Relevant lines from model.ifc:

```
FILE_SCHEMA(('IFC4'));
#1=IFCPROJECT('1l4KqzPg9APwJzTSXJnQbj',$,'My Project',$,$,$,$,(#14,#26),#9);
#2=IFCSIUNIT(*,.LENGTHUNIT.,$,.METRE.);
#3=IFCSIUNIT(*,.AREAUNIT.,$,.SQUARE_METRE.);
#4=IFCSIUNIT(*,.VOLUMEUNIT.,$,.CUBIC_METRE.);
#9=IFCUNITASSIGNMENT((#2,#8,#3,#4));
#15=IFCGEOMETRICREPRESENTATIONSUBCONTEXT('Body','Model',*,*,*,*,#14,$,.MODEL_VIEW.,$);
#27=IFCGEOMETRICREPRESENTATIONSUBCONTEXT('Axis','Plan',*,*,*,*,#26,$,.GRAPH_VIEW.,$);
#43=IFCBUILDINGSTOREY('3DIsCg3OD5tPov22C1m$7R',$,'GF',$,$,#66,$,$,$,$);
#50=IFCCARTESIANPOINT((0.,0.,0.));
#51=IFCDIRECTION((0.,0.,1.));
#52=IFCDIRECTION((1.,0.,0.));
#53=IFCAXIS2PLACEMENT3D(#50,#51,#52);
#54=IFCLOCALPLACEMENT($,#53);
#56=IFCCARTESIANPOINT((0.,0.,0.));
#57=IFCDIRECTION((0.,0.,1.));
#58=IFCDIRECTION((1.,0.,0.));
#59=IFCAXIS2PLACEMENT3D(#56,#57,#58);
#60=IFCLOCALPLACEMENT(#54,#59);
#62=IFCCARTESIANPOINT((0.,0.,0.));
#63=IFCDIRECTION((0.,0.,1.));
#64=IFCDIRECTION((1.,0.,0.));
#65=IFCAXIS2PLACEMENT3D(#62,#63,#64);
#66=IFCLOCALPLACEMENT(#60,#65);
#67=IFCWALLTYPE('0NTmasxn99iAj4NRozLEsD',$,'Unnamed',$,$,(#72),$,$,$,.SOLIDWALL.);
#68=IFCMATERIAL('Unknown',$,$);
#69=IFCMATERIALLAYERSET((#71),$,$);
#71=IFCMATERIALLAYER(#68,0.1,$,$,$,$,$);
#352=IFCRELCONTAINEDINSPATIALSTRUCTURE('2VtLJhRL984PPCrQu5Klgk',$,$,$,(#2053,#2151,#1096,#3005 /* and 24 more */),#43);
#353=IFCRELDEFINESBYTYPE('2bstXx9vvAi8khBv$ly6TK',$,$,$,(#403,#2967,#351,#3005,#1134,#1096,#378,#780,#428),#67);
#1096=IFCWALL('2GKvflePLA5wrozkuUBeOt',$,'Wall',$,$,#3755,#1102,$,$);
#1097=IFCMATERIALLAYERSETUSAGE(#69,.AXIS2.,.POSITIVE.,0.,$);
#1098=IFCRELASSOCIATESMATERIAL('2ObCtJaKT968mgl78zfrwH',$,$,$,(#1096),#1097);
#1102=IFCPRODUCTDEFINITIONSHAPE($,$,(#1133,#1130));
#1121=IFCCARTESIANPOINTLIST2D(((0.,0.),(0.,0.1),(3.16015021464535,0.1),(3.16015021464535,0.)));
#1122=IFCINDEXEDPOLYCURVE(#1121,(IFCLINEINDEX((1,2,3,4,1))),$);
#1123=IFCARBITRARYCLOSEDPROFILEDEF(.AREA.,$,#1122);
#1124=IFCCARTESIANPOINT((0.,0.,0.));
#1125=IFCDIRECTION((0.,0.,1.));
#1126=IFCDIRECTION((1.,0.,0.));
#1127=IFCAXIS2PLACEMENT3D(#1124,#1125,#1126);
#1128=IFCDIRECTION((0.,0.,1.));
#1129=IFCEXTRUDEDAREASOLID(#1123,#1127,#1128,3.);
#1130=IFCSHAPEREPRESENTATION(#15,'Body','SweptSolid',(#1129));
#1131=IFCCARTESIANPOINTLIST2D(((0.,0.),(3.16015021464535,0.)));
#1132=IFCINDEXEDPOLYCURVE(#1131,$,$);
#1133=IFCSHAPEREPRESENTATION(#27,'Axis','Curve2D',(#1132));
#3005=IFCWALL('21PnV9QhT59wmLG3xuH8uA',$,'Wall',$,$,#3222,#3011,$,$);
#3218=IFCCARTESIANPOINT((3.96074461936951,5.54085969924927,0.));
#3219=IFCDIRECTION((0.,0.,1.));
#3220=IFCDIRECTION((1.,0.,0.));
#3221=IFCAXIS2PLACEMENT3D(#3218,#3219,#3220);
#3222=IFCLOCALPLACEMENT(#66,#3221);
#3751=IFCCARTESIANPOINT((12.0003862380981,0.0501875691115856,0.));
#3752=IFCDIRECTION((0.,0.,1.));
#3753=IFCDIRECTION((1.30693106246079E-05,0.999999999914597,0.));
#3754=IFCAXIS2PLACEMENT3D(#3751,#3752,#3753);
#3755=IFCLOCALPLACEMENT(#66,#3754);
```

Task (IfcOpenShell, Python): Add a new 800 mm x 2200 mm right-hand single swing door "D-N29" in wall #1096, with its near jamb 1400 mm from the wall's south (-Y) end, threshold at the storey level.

```python
import numpy as np
import ifcopenshell
import ifcopenshell.api.feature
import ifcopenshell.api.geometry
import ifcopenshell.api.root
import ifcopenshell.api.spatial
import ifcopenshell.geom
import ifcopenshell.util.element
import ifcopenshell.util.placement
import ifcopenshell.util.representation
import ifcopenshell.util.shape
import ifcopenshell.util.unit

model = ifcopenshell.open("model.ifc")
unit_scale = ifcopenshell.util.unit.calculate_unit_scale(model)
settings = ifcopenshell.geom.settings()


def volume(element):
    """Net volume in cubic metres, openings subtracted."""
    shape = ifcopenshell.geom.create_shape(settings, element)
    return ifcopenshell.util.shape.get_volume(shape.geometry)


wall = model.by_id(1096)
storey = ifcopenshell.util.element.get_container(wall, ifc_class="IfcBuildingStorey")
context = ifcopenshell.util.representation.get_context(model, "Model", "Body", "MODEL_VIEW")
before = volume(wall)

width, height, from_end, sill = 0.8, 2.2, 1.4, 0.0  # metres

# The wall runs along its own X axis, and the end named is its -X end.
wall_shape = ifcopenshell.geom.create_shape(settings, wall)
x, y, z = ifcopenshell.util.shape.get_vertices(wall_shape.geometry).T
start = x.min() + from_end
face, thickness = float(y.min()), float(y.max() - y.min())
wall_matrix = ifcopenshell.util.placement.get_local_placement(wall.ObjectPlacement)
level = ifcopenshell.util.placement.get_local_placement(storey.ObjectPlacement)[2, 3]


def in_wall(x, y):
    """Placement at x, y metres in the wall's axes, at sill height."""
    matrix = wall_matrix.copy()
    matrix[:, 3] = wall_matrix @ np.array([x / unit_scale, y / unit_scale, 0.0, 1.0])
    matrix[2, 3] = level + sill / unit_scale
    return matrix


# Opening: a box that overshoots both wall faces by 50 mm.
opening = ifcopenshell.api.root.create_entity(model, ifc_class="IfcOpeningElement", predefined_type="OPENING")
box = ifcopenshell.api.geometry.add_wall_representation(
    model, context=context, length=width, height=height, thickness=thickness + 0.1
)
ifcopenshell.api.geometry.assign_representation(model, product=opening, representation=box)
ifcopenshell.api.geometry.edit_object_placement(model, product=opening, matrix=in_wall(start, face - 0.05), is_si=False)
ifcopenshell.api.feature.add_feature(model, feature=opening, element=wall)

door = ifcopenshell.api.root.create_entity(model, ifc_class="IfcDoor", name="D-N29", predefined_type="DOOR")
door.OverallWidth, door.OverallHeight = width / unit_scale, height / unit_scale
door.OperationType = "SINGLE_SWING_RIGHT"
body = ifcopenshell.api.geometry.add_door_representation(
    model,
    context=context,
    overall_width=door.OverallWidth,
    overall_height=door.OverallHeight,
    operation_type="SINGLE_SWING_RIGHT",
    lining_properties={"LiningDepth": thickness / unit_scale, "ThresholdDepth": thickness / unit_scale},
)
ifcopenshell.api.geometry.assign_representation(model, product=door, representation=body)
ifcopenshell.api.spatial.assign_container(model, products=[door], relating_structure=storey)
ifcopenshell.api.feature.add_filling(model, opening=opening, element=door)

# The lining spans the wall, so the door starts at the wall face.
ifcopenshell.api.geometry.edit_object_placement(model, product=door, matrix=in_wall(start, face), is_si=False)

after = volume(wall)

print(f"wall volume {before:.3f} -> {after:.3f} m3")

model.write("model_edited.ifc")
```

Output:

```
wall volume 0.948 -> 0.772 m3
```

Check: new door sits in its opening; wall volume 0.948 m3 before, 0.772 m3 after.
